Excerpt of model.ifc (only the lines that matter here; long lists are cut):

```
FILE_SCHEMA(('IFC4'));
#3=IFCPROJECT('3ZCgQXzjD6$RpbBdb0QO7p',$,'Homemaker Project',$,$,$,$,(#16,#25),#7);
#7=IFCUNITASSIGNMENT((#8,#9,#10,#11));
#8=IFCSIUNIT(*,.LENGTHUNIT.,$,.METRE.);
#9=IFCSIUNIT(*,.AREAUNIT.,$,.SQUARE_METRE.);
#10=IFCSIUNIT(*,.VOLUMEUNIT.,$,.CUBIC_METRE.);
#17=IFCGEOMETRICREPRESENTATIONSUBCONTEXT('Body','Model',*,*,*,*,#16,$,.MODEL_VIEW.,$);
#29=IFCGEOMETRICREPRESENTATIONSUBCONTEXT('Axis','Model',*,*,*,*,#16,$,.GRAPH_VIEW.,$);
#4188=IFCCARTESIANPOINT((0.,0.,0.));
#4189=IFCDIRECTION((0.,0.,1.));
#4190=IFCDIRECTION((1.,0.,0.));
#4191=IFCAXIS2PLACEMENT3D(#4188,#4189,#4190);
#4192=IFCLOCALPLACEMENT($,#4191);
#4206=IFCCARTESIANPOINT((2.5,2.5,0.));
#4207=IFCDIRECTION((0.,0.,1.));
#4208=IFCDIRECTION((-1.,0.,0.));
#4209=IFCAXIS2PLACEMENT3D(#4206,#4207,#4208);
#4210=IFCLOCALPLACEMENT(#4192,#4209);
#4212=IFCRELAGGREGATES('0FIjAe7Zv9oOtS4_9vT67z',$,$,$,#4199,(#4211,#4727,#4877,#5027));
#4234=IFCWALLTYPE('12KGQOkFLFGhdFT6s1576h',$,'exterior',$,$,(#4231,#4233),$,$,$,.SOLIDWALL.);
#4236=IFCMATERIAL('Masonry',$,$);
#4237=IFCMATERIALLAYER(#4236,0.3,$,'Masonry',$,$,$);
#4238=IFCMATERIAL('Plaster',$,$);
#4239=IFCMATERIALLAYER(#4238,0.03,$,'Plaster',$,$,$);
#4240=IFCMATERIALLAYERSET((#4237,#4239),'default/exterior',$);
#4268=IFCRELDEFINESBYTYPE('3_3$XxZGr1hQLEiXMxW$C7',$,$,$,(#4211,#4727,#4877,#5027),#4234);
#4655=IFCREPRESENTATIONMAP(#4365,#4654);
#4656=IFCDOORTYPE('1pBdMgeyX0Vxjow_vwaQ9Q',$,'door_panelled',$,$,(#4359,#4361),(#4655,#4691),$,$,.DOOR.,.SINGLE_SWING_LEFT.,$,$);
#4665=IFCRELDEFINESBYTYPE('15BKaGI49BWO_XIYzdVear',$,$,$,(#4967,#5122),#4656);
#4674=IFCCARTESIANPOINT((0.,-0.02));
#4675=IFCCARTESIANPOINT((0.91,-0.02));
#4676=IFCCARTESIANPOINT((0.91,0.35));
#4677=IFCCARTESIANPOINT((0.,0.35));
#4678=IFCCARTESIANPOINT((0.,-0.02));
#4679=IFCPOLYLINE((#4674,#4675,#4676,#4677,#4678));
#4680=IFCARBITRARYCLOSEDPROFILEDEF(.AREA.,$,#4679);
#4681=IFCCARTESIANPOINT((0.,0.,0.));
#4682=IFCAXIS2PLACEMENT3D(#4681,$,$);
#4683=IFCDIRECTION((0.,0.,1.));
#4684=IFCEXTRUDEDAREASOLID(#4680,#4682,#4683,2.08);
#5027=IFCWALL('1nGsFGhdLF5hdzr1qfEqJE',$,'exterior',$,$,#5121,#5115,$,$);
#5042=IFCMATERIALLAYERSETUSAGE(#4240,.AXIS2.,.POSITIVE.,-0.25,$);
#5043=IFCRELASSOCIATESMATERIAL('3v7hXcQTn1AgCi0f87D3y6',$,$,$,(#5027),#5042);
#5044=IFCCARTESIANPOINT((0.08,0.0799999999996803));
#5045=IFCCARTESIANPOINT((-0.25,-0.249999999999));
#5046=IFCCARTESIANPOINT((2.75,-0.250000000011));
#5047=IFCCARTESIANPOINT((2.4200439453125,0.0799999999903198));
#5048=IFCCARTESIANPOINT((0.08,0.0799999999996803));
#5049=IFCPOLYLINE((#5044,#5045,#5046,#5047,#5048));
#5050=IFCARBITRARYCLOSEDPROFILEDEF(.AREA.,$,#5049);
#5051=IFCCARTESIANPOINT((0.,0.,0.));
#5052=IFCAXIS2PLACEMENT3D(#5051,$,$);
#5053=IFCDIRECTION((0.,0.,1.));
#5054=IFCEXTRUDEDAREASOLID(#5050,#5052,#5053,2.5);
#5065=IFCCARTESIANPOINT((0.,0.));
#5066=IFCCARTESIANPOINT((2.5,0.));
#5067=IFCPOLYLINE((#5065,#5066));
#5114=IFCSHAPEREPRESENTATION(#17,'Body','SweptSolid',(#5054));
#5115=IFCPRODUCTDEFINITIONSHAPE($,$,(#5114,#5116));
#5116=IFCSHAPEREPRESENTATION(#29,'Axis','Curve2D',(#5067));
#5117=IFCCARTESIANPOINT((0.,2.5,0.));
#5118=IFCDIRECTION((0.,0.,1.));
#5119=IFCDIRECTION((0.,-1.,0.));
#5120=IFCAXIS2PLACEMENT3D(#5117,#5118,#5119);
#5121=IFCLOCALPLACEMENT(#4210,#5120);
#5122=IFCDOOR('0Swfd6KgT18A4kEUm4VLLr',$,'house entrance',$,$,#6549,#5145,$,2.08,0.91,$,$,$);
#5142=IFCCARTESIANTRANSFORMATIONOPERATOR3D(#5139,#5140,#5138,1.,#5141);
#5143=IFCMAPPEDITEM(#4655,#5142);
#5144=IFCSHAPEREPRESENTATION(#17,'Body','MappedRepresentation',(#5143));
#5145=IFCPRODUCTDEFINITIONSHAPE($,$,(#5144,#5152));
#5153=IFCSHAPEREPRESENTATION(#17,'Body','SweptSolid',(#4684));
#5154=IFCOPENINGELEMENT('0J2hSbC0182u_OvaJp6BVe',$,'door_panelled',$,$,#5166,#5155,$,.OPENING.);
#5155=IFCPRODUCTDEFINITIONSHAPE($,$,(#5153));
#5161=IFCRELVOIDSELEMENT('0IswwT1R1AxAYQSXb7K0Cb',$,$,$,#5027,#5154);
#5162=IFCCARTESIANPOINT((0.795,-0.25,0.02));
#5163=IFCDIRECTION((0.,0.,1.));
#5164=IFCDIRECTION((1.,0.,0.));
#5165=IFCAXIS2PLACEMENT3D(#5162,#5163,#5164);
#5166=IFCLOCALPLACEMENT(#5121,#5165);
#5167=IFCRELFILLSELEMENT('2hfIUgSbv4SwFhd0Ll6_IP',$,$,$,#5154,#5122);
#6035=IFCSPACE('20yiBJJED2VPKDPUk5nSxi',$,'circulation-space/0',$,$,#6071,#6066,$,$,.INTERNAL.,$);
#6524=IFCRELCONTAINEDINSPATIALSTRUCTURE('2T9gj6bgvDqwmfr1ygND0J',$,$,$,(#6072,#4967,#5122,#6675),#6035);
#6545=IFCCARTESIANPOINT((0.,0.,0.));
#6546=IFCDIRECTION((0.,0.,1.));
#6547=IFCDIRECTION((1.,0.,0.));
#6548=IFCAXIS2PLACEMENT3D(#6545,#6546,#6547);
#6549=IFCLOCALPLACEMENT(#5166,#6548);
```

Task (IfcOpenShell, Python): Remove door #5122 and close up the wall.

```python
import ifcopenshell
import ifcopenshell.api.feature
import ifcopenshell.api.root
import ifcopenshell.geom
import ifcopenshell.util.shape

model = ifcopenshell.open("model.ifc")
settings = ifcopenshell.geom.settings()


def volume(element):
    """Net volume in cubic metres, openings subtracted."""
    shape = ifcopenshell.geom.create_shape(settings, element)
    return ifcopenshell.util.shape.get_volume(shape.geometry)


door = model.by_guid("0Swfd6KgT18A4kEUm4VLLr")
opening = door.FillsVoids[0].RelatingOpeningElement
wall = opening.VoidsElements[0].RelatingBuildingElement
before = volume(wall)

ifcopenshell.api.root.remove_product(model, product=door)
ifcopenshell.api.feature.remove_feature(model, feature=opening)

after = volume(wall)

print(f"wall volume {before:.3f} -> {after:.3f} m3")

model.write("model_edited.ifc")
```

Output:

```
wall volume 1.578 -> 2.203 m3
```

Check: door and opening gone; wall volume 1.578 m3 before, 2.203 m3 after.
